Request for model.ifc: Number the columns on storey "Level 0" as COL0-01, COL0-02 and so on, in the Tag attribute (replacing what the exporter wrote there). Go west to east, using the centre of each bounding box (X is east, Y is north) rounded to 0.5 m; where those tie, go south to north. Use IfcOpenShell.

First a look at what the model holds.

```python
import ifcopenshell
import ifcopenshell.util.element
import ifcopenshell.util.placement

model = ifcopenshell.open("model.ifc")
print(model.schema)
storey = next(s for s in model.by_type("IfcBuildingStorey") if s.Name == "Level 0")
columns = [e for e in ifcopenshell.util.element.get_decomposition(storey) if e.is_a("IfcColumn")]
for e in sorted(columns, key=lambda e: e.id()):
    origin = ifcopenshell.util.placement.get_local_placement(e.ObjectPlacement)[:3, 3]
    print(e.id(), e.Tag, e.Name, origin.round(2) + 0.0, sep=" | ")
```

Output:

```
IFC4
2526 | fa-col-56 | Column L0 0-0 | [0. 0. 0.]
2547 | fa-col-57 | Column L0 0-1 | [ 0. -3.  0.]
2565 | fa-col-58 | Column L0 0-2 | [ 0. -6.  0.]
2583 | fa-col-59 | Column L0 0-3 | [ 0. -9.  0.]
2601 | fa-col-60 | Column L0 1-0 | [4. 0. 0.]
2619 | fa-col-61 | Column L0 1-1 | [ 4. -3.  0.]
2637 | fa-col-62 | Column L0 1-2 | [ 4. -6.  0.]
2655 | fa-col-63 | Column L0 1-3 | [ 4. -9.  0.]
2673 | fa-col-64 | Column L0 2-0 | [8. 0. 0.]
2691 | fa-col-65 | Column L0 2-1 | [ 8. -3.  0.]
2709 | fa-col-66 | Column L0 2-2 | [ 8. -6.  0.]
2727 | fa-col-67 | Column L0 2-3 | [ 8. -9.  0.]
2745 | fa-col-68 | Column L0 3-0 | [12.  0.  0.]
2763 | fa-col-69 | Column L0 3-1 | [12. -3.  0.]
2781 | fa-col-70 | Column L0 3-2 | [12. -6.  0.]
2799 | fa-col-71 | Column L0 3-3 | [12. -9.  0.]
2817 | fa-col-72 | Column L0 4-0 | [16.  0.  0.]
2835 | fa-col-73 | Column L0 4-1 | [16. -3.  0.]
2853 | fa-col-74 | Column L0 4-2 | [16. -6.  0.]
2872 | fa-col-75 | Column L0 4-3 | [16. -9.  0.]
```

```python
import ifcopenshell
import ifcopenshell.geom
import ifcopenshell.util.element
import ifcopenshell.util.shape

model = ifcopenshell.open("model.ifc")
settings = ifcopenshell.geom.settings()
settings.set("use-world-coords", True)


def centre(element):
    shape = ifcopenshell.geom.create_shape(settings, element)
    return ifcopenshell.util.shape.get_bbox_centroid(shape.geometry)


storey = next(s for s in model.by_type("IfcBuildingStorey") if s.Name == "Level 0")
columns = [e for e in ifcopenshell.util.element.get_decomposition(storey) if e.is_a("IfcColumn")]

# Insertion points can sit at a corner or the storey origin, so sort by the geometry (in metres).
centres = {e: centre(e) for e in columns}
columns.sort(key=lambda e: (round(centres[e][0] / 0.5), centres[e][1]))

for i, e in enumerate(columns, start=1):
    number = f"COL0-{i:02d}"
    e.Tag = number
    print(e.id(), number)

model.write("model_edited.ifc")
```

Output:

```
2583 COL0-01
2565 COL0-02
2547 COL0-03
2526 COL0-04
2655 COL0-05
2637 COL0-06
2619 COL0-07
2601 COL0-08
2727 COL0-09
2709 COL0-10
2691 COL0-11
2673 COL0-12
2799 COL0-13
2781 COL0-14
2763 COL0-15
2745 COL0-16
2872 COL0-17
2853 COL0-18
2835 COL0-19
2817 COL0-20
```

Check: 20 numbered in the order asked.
